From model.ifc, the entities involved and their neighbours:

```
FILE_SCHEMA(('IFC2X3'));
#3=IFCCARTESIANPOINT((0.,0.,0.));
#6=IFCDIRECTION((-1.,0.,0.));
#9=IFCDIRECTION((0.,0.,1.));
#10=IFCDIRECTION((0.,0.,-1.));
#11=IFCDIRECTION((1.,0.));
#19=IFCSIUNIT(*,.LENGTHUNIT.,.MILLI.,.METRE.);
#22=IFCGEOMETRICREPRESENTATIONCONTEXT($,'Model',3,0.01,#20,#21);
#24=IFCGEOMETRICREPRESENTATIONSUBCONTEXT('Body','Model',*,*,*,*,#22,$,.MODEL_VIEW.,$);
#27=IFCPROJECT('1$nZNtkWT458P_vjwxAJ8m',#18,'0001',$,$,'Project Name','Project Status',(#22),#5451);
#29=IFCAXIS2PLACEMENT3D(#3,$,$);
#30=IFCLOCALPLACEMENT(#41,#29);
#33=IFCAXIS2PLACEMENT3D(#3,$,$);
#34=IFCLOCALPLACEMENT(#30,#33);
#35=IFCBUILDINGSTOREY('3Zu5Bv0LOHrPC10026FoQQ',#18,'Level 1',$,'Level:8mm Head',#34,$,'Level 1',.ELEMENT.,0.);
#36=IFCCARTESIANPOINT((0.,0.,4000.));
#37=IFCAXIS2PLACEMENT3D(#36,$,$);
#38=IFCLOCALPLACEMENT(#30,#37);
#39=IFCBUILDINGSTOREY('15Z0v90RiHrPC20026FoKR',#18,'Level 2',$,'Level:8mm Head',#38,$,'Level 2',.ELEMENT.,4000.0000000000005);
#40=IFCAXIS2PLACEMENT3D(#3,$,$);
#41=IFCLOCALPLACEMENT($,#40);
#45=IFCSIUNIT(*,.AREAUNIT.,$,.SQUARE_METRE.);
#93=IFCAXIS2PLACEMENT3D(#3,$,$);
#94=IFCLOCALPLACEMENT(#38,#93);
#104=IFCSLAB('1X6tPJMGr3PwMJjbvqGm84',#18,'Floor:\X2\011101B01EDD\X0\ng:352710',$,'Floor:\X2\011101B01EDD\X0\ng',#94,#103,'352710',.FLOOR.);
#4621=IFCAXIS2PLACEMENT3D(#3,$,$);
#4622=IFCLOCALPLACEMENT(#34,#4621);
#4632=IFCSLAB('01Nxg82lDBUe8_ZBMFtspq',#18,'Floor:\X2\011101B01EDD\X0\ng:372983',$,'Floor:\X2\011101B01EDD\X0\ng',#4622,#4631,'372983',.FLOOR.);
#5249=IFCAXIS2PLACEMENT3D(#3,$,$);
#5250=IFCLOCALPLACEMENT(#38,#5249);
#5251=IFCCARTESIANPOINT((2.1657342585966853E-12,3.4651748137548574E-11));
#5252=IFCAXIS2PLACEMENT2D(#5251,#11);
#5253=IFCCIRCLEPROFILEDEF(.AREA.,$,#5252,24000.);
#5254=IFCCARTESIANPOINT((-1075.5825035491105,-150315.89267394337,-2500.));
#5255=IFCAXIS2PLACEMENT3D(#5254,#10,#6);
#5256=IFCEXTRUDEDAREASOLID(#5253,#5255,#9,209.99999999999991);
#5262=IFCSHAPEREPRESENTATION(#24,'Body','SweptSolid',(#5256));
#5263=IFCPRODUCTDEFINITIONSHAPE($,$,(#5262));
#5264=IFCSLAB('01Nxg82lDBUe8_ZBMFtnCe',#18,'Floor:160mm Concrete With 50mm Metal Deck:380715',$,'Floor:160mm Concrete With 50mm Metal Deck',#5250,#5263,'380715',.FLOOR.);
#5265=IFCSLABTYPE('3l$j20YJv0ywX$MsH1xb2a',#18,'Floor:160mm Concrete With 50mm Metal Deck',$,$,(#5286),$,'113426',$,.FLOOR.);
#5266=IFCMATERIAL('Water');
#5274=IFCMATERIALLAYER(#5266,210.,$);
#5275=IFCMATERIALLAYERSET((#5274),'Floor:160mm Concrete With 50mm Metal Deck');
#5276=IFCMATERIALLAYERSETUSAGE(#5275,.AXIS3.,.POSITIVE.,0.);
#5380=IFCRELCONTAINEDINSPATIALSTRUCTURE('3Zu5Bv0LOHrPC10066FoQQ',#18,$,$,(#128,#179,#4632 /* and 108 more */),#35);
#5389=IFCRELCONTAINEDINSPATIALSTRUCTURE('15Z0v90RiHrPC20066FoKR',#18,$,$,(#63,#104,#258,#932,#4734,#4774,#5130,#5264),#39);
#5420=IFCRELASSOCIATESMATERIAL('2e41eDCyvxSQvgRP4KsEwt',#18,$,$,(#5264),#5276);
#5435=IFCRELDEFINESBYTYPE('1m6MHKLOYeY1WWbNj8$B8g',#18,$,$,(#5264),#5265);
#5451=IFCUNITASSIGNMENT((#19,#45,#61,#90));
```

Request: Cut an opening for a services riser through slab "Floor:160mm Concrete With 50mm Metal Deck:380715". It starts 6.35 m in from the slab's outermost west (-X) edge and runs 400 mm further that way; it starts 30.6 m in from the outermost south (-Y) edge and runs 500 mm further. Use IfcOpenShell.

```python
import numpy as np
import ifcopenshell
import ifcopenshell.api.feature
import ifcopenshell.api.geometry
import ifcopenshell.api.root
import ifcopenshell.geom
import ifcopenshell.util.placement
import ifcopenshell.util.representation
import ifcopenshell.util.shape
import ifcopenshell.util.unit

model = ifcopenshell.open("model.ifc")
unit_scale = ifcopenshell.util.unit.calculate_unit_scale(model)
settings = ifcopenshell.geom.settings()


def volume(element):
    """Net volume in cubic metres, openings subtracted."""
    shape = ifcopenshell.geom.create_shape(settings, element)
    return ifcopenshell.util.shape.get_volume(shape.geometry)


slab = model.by_id(5264)
before = volume(slab)

# Extent in the slab's own axes, in metres. The edges named are its -X and -Y sides.
slab_shape = ifcopenshell.geom.create_shape(settings, slab)
vertices = ifcopenshell.util.shape.get_vertices(slab_shape.geometry)
x_min, y_min, bottom = vertices.min(axis=0)
top = vertices[:, 2].max()

opening = ifcopenshell.api.root.create_entity(model, ifc_class="IfcOpeningElement", name="Services riser opening")
context = ifcopenshell.util.representation.get_context(model, "Model", "Body", "MODEL_VIEW")
width, depth = 0.4, 0.5
outline = [(0.0, 0.0), (width, 0.0), (width, depth), (0.0, depth), (0.0, 0.0)]
# Overshoot both faces by 50 mm so the cut is clean.
shape = ifcopenshell.api.geometry.add_slab_representation(
    model, context=context, depth=top - bottom + 0.1, polyline=outline
)
ifcopenshell.api.geometry.assign_representation(model, product=opening, representation=shape)

matrix = ifcopenshell.util.placement.get_local_placement(slab.ObjectPlacement)
matrix[:, 3] = matrix @ np.append(np.array([x_min + 6.35, y_min + 30.6, bottom - 0.05]) / unit_scale, 1.0)
ifcopenshell.api.geometry.edit_object_placement(model, product=opening, matrix=matrix, is_si=False)
ifcopenshell.api.feature.add_feature(model, feature=opening, element=slab)

after = volume(slab)

print(f"slab volume {before:.3f} -> {after:.3f} m3")

model.write("model_updated.ifc")
```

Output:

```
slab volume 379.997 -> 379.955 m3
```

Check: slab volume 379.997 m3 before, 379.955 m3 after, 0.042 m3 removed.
